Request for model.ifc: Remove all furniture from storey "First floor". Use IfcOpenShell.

First a look at what the model holds.

```python
import ifcopenshell
import ifcopenshell.util.element

model = ifcopenshell.open("model.ifc")
print(model.schema)
storey = next(s for s in model.by_type("IfcBuildingStorey") if s.Name == "First floor")
furniture = [e for e in ifcopenshell.util.element.get_decomposition(storey) if e.is_a("IfcFurnishingElement")]
seen = {}
for e in furniture:
    element_type = ifcopenshell.util.element.get_type(e)
    name = element_type.Name if element_type not in (None, e) else None
    seen[name] = seen.get(name, 0) + 1
for name, count in sorted(seen.items(), key=str):
    print(count, "x", name)
```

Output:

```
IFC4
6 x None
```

```python
import ifcopenshell
import ifcopenshell.api.root
import ifcopenshell.util.element

model = ifcopenshell.open("model.ifc")

storey = next(s for s in model.by_type("IfcBuildingStorey") if s.Name == "First floor")
furniture = [e for e in ifcopenshell.util.element.get_decomposition(storey) if e.is_a("IfcFurnishingElement")]

for e in furniture:
    ifcopenshell.api.root.remove_product(model, product=e)
print(len(furniture), "removed")

model.write("model_v2.ifc")
```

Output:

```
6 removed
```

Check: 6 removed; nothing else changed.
